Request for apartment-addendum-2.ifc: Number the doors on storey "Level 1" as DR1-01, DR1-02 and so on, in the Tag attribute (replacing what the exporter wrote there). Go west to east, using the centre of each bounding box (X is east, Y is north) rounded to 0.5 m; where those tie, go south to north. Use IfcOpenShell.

First a look at what the model holds.

```python
import ifcopenshell
import ifcopenshell.util.element
import ifcopenshell.util.placement

model = ifcopenshell.open("apartment-addendum-2.ifc")
print(model.schema)
storey = next(s for s in model.by_type("IfcBuildingStorey") if s.Name == "Level 1")
doors = [e for e in ifcopenshell.util.element.get_decomposition(storey) if e.is_a("IfcDoor")]
for e in sorted(doors, key=lambda e: e.id()):
    origin = ifcopenshell.util.placement.get_local_placement(e.ObjectPlacement)[:3, 3]
    print(e.id(), e.Tag, e.Name, origin.round(2) + 0.0, sep=" | ")
```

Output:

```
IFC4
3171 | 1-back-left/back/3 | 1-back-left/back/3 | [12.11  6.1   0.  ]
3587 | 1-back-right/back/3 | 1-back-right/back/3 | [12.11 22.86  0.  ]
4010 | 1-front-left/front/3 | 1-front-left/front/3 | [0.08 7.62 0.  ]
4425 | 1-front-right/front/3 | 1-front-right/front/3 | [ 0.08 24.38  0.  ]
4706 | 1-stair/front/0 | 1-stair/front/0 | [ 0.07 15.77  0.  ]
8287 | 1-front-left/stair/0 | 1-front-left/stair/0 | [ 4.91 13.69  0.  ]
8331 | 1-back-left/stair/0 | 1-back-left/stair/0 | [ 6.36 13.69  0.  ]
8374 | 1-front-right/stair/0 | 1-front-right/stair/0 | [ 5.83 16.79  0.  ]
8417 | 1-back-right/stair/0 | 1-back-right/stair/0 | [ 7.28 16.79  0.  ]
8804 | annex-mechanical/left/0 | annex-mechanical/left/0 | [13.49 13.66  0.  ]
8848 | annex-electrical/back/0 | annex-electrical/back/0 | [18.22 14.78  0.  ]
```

```python
import ifcopenshell
import ifcopenshell.geom
import ifcopenshell.util.element
import ifcopenshell.util.shape

model = ifcopenshell.open("apartment-addendum-2.ifc")
settings = ifcopenshell.geom.settings()
settings.set("use-world-coords", True)


def centre(element):
    shape = ifcopenshell.geom.create_shape(settings, element)
    return ifcopenshell.util.shape.get_bbox_centroid(shape.geometry)


storey = next(s for s in model.by_type("IfcBuildingStorey") if s.Name == "Level 1")
doors = [e for e in ifcopenshell.util.element.get_decomposition(storey) if e.is_a("IfcDoor")]

# Insertion points can sit at a corner or the storey origin, so sort by the geometry (in metres).
centres = {e: centre(e) for e in doors}
doors.sort(key=lambda e: (round(centres[e][0] / 0.5), centres[e][1]))

for i, e in enumerate(doors, start=1):
    number = f"DR1-{i:02d}"
    e.Tag = number
    print(e.id(), number)

model.write("apartment-addendum-2_v2.ifc")
```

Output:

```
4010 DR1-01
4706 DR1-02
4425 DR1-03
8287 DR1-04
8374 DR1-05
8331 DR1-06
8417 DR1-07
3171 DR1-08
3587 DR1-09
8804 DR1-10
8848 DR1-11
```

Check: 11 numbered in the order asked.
